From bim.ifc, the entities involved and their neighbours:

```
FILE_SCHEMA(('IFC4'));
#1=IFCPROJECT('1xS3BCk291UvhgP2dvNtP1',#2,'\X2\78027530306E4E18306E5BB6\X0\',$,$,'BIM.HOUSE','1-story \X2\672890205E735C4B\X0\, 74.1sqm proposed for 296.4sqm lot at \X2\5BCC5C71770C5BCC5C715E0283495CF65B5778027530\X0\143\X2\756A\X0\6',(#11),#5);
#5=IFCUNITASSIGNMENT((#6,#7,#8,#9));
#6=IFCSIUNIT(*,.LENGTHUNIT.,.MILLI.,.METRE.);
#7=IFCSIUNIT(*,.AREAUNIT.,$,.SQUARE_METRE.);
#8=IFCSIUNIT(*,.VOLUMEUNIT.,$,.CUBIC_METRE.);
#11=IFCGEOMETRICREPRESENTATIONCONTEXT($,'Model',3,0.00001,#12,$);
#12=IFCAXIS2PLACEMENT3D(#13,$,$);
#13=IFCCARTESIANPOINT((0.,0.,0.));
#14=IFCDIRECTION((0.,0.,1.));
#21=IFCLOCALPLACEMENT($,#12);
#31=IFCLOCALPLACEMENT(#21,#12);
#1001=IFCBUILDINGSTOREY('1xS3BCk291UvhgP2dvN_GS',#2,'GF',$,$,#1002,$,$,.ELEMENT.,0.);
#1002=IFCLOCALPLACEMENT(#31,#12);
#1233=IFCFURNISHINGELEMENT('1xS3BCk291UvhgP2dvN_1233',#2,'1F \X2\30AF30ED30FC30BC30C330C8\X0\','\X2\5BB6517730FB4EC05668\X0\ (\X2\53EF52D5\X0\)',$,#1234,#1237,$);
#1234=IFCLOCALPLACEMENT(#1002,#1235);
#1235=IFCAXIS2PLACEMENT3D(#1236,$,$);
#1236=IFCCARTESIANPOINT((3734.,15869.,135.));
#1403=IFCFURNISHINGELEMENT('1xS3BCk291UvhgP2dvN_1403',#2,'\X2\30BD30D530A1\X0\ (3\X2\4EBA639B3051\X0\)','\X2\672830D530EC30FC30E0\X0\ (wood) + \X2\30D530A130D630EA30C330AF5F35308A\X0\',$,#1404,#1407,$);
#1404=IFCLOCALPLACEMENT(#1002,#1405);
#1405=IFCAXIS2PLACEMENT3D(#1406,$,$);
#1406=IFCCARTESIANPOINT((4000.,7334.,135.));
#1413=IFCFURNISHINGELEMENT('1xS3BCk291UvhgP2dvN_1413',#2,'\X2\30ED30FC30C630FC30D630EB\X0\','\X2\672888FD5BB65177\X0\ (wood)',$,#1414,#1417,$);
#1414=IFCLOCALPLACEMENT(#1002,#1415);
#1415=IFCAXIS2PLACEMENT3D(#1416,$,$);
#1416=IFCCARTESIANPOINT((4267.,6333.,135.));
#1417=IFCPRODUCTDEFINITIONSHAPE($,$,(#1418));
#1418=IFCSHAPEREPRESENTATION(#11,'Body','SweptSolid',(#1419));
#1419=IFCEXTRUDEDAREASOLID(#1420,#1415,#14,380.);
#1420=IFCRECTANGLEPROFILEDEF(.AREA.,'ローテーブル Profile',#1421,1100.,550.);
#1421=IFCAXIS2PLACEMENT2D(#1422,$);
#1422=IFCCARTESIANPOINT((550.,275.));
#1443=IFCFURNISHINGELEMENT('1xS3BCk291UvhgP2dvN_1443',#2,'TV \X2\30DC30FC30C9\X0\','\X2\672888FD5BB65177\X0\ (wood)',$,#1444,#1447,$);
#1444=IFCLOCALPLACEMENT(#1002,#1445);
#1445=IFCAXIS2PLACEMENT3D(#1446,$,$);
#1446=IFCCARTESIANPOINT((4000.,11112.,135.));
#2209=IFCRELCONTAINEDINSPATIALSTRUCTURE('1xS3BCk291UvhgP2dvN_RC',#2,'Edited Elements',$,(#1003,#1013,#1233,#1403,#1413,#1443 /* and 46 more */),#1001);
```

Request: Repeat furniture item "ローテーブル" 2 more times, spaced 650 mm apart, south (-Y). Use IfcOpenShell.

```python
import numpy as np
import ifcopenshell
import ifcopenshell.api.geometry
import ifcopenshell.api.root
import ifcopenshell.util.element
import ifcopenshell.util.placement
import ifcopenshell.util.unit

model = ifcopenshell.open("bim.ifc")
unit_scale = ifcopenshell.util.unit.calculate_unit_scale(model)


def reuse_history(source, copy):
    """copy_class also copies each property set's owner history, people and application; keep the originals."""
    for rel in copy.IsDefinedBy:
        if rel.is_a("IfcRelDefinesByProperties") and (history := rel.RelatingPropertyDefinition.OwnerHistory):
            rel.RelatingPropertyDefinition.OwnerHistory = source.OwnerHistory
            ifcopenshell.util.element.remove_deep2(model, history)


source = model.by_guid("1xS3BCk291UvhgP2dvN_1413")
base = ifcopenshell.util.placement.get_local_placement(source.ObjectPlacement)
step = np.array([0.0, -1.0, 0.0]) * 0.65 / unit_scale

for i in range(1, 3):
    copy = ifcopenshell.api.root.copy_class(model, product=source)
    copy.Representation = ifcopenshell.util.element.copy_deep(
        model, source.Representation, exclude=["IfcGeometricRepresentationContext", "IfcRepresentationMap"]
    )
    reuse_history(source, copy)
    matrix = base.copy()
    matrix[:3, 3] += i * step
    print("added at", matrix[:3, 3].round(3) + 0.0)
    ifcopenshell.api.geometry.edit_object_placement(model, product=copy, matrix=matrix, is_si=False)

model.write("bim_rev.ifc")
```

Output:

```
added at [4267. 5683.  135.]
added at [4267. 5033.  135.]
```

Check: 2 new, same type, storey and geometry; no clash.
